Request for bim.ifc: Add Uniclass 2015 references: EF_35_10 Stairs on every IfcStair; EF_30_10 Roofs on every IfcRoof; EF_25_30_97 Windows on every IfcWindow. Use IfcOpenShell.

First a look at what the model holds.

```python
import ifcopenshell

model = ifcopenshell.open("bim.ifc")
print(model.schema)
print("classifications:", [c.Name for c in model.by_type("IfcClassification")])
for ifc_class in ("IfcDoor", "IfcRoof", "IfcStair", "IfcWall", "IfcWindow"):
    print(ifc_class, len(model.by_type(ifc_class)))
```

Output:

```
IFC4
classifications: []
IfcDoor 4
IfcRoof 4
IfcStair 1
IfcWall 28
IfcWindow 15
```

```python
import ifcopenshell
import ifcopenshell.api.classification

model = ifcopenshell.open("bim.ifc")

system = ifcopenshell.api.classification.add_classification(model, classification="Uniclass 2015")

codes = {
    "IfcStair": ("EF_35_10", "Stairs"),
    "IfcRoof": ("EF_30_10", "Roofs"),
    "IfcWindow": ("EF_25_30_97", "Windows"),
}
for ifc_class, (code, name) in codes.items():
    products = model.by_type(ifc_class)
    ifcopenshell.api.classification.add_reference(
        model, products=products, classification=system, identification=code, name=name
    )
    print(code, len(products))

model.write("bim_v2.ifc")
```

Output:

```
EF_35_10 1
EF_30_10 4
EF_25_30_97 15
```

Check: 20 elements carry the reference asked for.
